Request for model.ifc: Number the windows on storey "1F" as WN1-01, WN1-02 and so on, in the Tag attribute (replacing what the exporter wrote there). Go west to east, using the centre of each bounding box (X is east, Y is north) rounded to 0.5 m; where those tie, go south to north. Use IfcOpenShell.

First a look at what the model holds.

```python
import ifcopenshell
import ifcopenshell.util.element
import ifcopenshell.util.placement

model = ifcopenshell.open("model.ifc")
print(model.schema)
storey = next(s for s in model.by_type("IfcBuildingStorey") if s.Name == "1F")
windows = [e for e in ifcopenshell.util.element.get_decomposition(storey) if e.is_a("IfcWindow")]
for e in sorted(windows, key=lambda e: e.id()):
    origin = ifcopenshell.util.placement.get_local_placement(e.ObjectPlacement)[:3, 3]
    print(e.id(), e.Tag, e.Name, origin.round(2) + 0.0, sep=" | ")
```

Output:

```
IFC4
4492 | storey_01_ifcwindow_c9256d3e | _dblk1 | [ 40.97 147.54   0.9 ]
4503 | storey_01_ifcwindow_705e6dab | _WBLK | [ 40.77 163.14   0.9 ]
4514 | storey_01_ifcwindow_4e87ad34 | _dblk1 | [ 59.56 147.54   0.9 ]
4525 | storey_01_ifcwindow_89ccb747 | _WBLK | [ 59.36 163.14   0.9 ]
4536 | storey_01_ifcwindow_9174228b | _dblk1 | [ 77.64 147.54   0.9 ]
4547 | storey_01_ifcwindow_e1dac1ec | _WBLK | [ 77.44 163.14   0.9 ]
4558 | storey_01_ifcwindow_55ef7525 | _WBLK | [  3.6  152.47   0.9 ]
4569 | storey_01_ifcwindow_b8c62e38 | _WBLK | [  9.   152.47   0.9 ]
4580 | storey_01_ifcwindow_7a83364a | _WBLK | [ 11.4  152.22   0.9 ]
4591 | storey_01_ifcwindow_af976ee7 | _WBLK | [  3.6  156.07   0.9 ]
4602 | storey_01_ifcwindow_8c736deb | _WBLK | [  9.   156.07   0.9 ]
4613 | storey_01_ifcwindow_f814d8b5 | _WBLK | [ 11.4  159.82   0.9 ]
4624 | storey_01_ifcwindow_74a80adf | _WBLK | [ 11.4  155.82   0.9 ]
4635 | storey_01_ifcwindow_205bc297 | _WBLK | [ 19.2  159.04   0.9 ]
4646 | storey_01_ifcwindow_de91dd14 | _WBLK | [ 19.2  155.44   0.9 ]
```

```python
import ifcopenshell
import ifcopenshell.geom
import ifcopenshell.util.element
import ifcopenshell.util.shape

model = ifcopenshell.open("model.ifc")
settings = ifcopenshell.geom.settings()
settings.set("use-world-coords", True)


def centre(element):
    shape = ifcopenshell.geom.create_shape(settings, element)
    return ifcopenshell.util.shape.get_bbox_centroid(shape.geometry)


storey = next(s for s in model.by_type("IfcBuildingStorey") if s.Name == "1F")
windows = [e for e in ifcopenshell.util.element.get_decomposition(storey) if e.is_a("IfcWindow")]

# Insertion points can sit at a corner or the storey origin, so sort by the geometry (in metres).
centres = {e: centre(e) for e in windows}
windows.sort(key=lambda e: (round(centres[e][0] / 0.5), centres[e][1]))

for i, e in enumerate(windows, start=1):
    number = f"WN1-{i:02d}"
    e.Tag = number
    print(e.id(), number)

model.write("model_updated.ifc")
```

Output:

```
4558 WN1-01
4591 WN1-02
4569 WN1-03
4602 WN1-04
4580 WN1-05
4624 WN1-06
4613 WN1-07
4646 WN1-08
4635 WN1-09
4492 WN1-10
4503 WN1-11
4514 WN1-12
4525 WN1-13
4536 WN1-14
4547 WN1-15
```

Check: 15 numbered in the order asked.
